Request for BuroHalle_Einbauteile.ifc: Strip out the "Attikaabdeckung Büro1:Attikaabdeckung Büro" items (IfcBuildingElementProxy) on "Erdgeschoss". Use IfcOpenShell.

First a look at what the model holds.

```python
import ifcopenshell
import ifcopenshell.util.element

model = ifcopenshell.open("BuroHalle_Einbauteile.ifc")
print(model.schema)
storey = next(s for s in model.by_type("IfcBuildingStorey") if s.Name == "Erdgeschoss")
proxies = [e for e in ifcopenshell.util.element.get_decomposition(storey) if e.is_a("IfcBuildingElementProxy")]
seen = {}
for e in proxies:
    element_type = ifcopenshell.util.element.get_type(e)
    name = element_type.Name if element_type not in (None, e) else None
    seen[name] = seen.get(name, 0) + 1
for name, count in sorted(seen.items(), key=str):
    print(count, "x", name)
```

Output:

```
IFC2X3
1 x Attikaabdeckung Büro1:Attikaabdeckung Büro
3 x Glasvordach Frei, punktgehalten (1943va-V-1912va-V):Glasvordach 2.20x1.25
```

```python
import ifcopenshell
import ifcopenshell.api.root
import ifcopenshell.util.element

model = ifcopenshell.open("BuroHalle_Einbauteile.ifc")

storey = next(s for s in model.by_type("IfcBuildingStorey") if s.Name == "Erdgeschoss")
proxies = [e for e in ifcopenshell.util.element.get_decomposition(storey) if e.is_a("IfcBuildingElementProxy")]
targets = [e for e in proxies if (t := ifcopenshell.util.element.get_type(e)) not in (None, e) and t.Name == "Attikaabdeckung Büro1:Attikaabdeckung Büro"]

for e in targets:
    ifcopenshell.api.root.remove_product(model, product=e)
print(len(targets), "removed")

model.write("BuroHalle_Einbauteile-out.ifc")
```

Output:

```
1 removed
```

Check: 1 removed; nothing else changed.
